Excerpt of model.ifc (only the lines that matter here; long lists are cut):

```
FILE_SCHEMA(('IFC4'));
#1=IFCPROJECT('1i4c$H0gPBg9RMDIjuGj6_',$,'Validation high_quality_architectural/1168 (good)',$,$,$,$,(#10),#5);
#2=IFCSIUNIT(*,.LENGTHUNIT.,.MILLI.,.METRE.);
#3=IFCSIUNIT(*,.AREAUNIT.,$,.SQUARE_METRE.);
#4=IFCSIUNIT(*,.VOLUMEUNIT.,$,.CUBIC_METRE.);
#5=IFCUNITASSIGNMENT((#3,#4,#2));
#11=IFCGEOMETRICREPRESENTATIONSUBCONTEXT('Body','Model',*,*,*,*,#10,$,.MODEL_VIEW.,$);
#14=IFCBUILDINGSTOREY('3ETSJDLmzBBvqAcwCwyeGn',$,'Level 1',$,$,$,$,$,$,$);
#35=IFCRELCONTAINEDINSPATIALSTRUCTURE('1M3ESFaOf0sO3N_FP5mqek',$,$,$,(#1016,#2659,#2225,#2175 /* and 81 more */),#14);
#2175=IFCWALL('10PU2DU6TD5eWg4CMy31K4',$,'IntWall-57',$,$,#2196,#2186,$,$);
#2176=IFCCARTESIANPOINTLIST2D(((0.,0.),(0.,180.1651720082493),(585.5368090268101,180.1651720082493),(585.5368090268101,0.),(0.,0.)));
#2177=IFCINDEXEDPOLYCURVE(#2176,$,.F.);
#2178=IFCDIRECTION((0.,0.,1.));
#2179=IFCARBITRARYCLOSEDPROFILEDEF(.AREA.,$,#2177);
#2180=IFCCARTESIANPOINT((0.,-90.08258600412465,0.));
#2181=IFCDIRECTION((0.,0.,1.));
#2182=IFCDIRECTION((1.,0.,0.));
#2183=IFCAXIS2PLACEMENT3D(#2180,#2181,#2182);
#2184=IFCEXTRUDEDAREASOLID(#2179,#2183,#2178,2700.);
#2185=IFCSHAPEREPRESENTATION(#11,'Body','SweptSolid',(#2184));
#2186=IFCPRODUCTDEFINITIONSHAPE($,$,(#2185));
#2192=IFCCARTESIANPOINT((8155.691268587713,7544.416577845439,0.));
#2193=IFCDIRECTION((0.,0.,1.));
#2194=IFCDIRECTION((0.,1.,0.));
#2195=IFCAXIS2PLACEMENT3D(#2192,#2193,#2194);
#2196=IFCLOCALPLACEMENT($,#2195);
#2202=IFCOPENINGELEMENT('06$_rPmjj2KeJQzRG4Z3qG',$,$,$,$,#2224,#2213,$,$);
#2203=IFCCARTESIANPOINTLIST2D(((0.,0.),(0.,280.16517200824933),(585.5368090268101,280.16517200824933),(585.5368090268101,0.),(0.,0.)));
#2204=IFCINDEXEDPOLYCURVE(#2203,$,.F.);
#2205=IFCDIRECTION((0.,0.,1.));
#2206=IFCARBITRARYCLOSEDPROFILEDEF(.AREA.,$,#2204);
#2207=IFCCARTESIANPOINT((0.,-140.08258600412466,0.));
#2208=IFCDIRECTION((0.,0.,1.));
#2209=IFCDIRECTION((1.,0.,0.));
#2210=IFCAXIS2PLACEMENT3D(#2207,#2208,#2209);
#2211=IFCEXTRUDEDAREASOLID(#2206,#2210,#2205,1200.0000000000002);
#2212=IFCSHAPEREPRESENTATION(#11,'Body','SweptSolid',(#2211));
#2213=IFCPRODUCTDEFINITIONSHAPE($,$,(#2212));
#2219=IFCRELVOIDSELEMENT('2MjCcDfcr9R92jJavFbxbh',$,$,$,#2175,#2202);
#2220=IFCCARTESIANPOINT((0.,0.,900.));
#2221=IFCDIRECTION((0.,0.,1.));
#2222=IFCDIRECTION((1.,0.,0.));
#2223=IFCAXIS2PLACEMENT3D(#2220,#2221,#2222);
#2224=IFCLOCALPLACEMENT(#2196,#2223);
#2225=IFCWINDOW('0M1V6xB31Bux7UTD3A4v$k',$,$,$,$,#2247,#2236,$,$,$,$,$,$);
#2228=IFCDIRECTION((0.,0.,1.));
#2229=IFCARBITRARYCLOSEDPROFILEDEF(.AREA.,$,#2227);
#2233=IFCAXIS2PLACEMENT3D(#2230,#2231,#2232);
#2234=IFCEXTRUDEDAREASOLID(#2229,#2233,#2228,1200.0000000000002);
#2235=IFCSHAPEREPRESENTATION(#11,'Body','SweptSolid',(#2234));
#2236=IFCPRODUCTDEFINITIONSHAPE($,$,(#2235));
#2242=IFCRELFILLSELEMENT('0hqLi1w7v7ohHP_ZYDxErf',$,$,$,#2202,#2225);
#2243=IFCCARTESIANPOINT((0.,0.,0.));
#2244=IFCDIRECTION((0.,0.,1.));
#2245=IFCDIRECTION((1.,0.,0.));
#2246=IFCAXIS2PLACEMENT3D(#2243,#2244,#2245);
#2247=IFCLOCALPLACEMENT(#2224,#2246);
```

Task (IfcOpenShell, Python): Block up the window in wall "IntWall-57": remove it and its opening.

```python
import ifcopenshell
import ifcopenshell.api.feature
import ifcopenshell.api.root
import ifcopenshell.geom
import ifcopenshell.util.shape

model = ifcopenshell.open("model.ifc")
settings = ifcopenshell.geom.settings()


def volume(element):
    """Net volume in cubic metres, openings subtracted."""
    shape = ifcopenshell.geom.create_shape(settings, element)
    return ifcopenshell.util.shape.get_volume(shape.geometry)


window = model.by_id(2225)
opening = window.FillsVoids[0].RelatingOpeningElement
wall = opening.VoidsElements[0].RelatingBuildingElement
before = volume(wall)

ifcopenshell.api.root.remove_product(model, product=window)
ifcopenshell.api.feature.remove_feature(model, feature=opening)

after = volume(wall)

print(f"wall volume {before:.3f} -> {after:.3f} m3")

model.write("model_v2.ifc")
```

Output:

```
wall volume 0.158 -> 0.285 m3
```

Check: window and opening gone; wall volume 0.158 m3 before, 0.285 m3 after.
